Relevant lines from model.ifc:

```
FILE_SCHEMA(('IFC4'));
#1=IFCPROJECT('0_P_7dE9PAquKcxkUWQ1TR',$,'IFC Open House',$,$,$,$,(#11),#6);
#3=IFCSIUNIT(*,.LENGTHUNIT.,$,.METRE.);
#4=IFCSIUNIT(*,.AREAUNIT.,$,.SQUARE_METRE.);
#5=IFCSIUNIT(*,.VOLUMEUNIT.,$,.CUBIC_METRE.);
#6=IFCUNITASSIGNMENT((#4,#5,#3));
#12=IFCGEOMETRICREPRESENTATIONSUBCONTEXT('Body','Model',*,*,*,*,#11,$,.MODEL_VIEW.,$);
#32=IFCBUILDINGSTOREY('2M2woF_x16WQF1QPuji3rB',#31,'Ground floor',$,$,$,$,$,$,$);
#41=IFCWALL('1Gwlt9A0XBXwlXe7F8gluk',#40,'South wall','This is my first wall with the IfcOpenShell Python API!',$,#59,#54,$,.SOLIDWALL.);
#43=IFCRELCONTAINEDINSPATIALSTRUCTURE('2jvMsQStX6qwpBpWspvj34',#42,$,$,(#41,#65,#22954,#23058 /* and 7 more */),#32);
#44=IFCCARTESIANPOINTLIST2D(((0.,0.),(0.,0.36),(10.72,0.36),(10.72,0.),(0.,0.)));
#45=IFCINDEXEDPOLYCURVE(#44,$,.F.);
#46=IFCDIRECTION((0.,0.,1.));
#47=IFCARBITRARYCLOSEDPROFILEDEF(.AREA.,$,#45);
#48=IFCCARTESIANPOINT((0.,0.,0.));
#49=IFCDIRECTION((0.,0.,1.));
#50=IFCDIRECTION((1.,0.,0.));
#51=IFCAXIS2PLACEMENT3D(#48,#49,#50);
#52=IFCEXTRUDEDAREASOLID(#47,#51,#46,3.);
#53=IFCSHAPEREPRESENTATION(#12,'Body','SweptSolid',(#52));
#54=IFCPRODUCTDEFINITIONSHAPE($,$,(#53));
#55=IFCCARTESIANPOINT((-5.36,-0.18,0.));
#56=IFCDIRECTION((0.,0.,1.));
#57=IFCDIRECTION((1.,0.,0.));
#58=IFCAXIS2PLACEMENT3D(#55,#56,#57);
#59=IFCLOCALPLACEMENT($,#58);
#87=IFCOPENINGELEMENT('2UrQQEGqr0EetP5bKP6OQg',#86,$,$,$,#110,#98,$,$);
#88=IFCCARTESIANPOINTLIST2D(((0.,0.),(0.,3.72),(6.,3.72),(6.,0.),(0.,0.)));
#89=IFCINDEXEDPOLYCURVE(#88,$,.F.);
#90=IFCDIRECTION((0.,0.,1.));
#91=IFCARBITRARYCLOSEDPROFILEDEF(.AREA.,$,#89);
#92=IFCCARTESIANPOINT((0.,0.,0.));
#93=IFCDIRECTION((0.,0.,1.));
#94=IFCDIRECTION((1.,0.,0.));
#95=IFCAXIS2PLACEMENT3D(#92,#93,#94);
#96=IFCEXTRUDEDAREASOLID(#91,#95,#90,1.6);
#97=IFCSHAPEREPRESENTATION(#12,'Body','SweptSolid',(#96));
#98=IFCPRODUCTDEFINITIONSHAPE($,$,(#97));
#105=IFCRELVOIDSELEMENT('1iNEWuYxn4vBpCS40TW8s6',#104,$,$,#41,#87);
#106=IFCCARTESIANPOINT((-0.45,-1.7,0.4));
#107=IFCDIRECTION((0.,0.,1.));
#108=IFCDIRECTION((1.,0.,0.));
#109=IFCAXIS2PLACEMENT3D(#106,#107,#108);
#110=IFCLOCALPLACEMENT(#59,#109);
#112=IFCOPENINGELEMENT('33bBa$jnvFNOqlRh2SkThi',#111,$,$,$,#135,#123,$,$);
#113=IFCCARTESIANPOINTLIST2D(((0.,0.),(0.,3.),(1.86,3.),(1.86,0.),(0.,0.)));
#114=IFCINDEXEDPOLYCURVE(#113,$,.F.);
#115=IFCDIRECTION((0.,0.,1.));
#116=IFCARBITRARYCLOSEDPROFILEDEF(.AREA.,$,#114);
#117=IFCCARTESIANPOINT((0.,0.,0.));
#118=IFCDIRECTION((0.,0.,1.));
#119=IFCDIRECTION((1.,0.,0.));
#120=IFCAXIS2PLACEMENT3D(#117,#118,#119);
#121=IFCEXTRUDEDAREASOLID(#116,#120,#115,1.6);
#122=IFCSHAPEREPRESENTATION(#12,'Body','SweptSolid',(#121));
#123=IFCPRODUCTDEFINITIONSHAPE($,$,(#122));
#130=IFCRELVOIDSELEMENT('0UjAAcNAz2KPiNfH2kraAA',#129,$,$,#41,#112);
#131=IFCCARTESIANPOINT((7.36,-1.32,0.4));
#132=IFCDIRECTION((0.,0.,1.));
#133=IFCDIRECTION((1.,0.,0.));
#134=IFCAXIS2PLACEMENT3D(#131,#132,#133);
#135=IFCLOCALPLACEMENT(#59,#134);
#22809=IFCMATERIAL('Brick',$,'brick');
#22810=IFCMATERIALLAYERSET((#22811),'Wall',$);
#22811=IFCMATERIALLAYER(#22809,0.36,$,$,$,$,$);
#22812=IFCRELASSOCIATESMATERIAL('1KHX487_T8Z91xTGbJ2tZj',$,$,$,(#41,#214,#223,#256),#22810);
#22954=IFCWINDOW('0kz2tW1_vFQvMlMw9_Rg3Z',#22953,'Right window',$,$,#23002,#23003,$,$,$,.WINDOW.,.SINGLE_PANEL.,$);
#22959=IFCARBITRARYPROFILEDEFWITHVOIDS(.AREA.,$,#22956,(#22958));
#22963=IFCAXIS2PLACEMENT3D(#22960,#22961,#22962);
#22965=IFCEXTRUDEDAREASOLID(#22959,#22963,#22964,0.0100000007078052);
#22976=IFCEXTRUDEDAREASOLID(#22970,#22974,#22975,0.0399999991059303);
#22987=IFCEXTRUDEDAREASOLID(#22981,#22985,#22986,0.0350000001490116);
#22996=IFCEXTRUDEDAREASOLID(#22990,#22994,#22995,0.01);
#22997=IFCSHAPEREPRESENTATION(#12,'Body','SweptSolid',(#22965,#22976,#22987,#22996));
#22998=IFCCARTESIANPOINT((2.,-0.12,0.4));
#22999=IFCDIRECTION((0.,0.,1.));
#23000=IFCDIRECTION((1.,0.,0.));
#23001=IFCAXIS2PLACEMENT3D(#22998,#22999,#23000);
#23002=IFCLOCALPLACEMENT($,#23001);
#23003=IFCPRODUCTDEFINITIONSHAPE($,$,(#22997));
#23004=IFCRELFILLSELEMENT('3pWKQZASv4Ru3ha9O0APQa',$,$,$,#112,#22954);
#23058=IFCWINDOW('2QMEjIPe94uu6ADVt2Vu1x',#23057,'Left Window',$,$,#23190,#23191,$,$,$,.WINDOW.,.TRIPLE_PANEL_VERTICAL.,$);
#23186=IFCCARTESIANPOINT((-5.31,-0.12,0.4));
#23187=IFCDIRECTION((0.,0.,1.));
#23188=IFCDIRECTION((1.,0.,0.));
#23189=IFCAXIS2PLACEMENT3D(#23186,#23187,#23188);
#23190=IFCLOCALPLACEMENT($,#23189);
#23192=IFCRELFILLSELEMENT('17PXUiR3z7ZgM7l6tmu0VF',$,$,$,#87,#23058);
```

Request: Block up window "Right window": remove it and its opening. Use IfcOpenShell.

```python
import ifcopenshell
import ifcopenshell.api.feature
import ifcopenshell.api.root
import ifcopenshell.geom
import ifcopenshell.util.shape

model = ifcopenshell.open("model.ifc")
settings = ifcopenshell.geom.settings()


def volume(element):
    """Net volume in cubic metres, openings subtracted."""
    shape = ifcopenshell.geom.create_shape(settings, element)
    return ifcopenshell.util.shape.get_volume(shape.geometry)


window = model.by_id(22954)
opening = window.FillsVoids[0].RelatingOpeningElement
wall = opening.VoidsElements[0].RelatingBuildingElement
before = volume(wall)

ifcopenshell.api.root.remove_product(model, product=window)
ifcopenshell.api.feature.remove_feature(model, feature=opening)

after = volume(wall)

print(f"wall volume {before:.3f} -> {after:.3f} m3")

model.write("model_v2.ifc")
```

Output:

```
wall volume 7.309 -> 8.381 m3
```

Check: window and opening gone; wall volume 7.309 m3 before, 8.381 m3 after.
